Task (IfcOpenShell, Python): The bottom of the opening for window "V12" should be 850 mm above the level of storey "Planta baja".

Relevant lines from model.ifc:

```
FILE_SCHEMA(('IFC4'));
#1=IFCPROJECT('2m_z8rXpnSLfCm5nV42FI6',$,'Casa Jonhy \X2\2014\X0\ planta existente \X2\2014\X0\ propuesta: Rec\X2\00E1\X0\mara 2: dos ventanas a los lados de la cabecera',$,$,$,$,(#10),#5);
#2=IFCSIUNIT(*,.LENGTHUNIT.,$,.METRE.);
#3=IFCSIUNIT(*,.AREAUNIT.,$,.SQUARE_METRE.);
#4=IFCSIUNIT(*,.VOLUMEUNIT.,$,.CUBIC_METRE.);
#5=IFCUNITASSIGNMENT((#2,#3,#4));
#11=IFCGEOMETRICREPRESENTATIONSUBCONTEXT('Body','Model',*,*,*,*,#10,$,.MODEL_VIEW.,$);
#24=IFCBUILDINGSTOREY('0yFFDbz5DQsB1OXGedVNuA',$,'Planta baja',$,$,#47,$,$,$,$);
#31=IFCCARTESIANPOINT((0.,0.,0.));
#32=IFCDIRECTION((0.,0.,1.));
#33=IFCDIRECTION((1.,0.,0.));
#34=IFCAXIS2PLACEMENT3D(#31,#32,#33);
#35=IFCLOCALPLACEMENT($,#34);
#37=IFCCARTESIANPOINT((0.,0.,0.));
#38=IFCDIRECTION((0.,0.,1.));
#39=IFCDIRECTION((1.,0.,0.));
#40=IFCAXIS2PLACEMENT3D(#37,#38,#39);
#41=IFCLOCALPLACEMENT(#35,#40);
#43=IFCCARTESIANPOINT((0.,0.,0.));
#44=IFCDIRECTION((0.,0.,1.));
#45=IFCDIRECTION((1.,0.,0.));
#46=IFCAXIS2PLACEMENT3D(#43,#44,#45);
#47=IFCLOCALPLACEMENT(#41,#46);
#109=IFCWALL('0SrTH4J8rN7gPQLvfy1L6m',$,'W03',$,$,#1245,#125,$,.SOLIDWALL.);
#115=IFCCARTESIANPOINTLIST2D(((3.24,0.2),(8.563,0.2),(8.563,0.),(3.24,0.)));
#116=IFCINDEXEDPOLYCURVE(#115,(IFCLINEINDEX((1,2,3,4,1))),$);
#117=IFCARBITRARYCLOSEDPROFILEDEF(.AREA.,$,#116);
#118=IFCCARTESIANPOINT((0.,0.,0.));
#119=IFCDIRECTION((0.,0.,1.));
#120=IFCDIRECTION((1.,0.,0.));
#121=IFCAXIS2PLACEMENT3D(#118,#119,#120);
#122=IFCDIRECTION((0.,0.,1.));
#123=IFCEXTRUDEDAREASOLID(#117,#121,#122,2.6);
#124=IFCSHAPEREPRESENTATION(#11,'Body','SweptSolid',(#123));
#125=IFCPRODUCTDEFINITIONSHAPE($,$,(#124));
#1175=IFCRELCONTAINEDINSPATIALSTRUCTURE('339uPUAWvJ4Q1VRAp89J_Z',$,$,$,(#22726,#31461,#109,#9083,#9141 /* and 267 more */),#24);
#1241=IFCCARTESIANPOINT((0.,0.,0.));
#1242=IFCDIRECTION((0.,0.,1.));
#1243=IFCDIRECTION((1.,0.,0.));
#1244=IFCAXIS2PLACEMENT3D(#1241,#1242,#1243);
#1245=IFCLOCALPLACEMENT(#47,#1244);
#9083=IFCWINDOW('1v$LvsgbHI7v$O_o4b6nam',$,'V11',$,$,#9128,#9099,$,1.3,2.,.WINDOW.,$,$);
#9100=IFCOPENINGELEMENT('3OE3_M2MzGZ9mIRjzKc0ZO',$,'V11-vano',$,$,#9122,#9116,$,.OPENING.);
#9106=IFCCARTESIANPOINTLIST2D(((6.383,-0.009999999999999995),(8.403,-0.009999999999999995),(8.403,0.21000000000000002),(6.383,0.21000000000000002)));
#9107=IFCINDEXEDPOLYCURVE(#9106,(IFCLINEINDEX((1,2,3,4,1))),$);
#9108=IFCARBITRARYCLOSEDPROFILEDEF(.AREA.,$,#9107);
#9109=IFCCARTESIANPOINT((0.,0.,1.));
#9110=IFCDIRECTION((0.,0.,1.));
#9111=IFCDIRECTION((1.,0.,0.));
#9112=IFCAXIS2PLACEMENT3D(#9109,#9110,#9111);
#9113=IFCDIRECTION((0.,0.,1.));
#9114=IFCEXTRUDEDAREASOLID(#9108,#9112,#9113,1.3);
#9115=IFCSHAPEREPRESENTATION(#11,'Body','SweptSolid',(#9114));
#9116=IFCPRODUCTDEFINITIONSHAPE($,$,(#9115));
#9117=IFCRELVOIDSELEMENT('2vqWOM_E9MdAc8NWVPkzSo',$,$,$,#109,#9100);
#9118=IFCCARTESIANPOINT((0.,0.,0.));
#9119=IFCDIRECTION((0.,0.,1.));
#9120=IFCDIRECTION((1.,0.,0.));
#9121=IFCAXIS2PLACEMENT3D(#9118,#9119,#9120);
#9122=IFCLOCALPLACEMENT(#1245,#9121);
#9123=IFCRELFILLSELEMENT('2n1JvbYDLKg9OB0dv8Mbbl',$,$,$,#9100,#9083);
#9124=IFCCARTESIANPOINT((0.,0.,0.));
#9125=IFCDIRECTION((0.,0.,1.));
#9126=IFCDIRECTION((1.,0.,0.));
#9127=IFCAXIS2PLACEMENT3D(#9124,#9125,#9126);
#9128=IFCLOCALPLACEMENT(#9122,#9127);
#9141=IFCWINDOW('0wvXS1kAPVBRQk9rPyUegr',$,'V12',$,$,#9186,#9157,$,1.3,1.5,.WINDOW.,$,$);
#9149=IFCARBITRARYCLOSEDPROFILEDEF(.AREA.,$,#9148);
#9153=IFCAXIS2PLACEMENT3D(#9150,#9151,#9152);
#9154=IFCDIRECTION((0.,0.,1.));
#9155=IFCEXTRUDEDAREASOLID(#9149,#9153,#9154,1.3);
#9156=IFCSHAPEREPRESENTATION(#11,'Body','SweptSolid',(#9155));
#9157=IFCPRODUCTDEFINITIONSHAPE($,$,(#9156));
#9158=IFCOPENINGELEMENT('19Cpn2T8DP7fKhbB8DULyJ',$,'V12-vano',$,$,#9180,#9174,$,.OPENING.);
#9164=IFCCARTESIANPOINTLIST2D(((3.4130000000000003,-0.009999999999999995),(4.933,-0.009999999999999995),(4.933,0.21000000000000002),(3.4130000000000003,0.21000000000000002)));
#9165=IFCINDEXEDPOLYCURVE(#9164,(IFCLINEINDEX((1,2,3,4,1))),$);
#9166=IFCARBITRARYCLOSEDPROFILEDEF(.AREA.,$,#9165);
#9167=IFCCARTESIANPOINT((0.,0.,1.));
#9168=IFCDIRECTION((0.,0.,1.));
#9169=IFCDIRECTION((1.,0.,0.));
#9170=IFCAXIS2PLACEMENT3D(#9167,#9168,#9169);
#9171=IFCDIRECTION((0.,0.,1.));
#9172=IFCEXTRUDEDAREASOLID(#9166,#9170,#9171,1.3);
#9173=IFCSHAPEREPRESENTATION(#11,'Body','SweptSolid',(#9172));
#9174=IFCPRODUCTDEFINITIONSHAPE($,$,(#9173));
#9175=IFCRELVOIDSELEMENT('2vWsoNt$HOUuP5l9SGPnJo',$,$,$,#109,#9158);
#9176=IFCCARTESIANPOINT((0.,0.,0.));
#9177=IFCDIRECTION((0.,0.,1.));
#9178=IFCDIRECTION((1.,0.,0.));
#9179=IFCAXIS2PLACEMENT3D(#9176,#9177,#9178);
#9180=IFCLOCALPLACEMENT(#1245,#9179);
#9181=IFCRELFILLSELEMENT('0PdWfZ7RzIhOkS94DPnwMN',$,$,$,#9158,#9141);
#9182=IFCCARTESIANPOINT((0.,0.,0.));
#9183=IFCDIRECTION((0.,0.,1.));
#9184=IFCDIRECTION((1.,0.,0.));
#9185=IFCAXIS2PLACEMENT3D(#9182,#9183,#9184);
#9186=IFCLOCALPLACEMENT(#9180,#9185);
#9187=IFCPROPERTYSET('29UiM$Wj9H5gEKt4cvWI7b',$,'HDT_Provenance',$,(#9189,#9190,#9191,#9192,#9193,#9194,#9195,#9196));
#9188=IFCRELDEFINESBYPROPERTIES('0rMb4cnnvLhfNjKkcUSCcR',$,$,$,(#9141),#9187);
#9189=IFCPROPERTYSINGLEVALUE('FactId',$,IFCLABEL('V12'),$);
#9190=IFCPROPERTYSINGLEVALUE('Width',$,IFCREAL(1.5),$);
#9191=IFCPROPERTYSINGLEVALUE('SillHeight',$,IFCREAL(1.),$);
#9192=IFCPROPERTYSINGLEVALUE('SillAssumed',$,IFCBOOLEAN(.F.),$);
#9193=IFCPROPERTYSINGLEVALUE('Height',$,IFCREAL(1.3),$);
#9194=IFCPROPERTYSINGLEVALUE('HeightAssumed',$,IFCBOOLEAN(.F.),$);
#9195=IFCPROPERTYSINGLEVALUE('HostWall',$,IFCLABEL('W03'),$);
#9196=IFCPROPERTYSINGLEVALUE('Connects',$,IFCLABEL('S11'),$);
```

```python
import numpy as np
import ifcopenshell
import ifcopenshell.api.geometry
import ifcopenshell.api.pset
import ifcopenshell.geom
import ifcopenshell.util.element
import ifcopenshell.util.placement
import ifcopenshell.util.shape
import ifcopenshell.util.unit

model = ifcopenshell.open("model.ifc")
unit_scale = ifcopenshell.util.unit.calculate_unit_scale(model)

window = model.by_id(9141)
opening = window.FillsVoids[0].RelatingOpeningElement
storey = ifcopenshell.util.element.get_container(window, ifc_class="IfcBuildingStorey")
level = ifcopenshell.util.placement.get_local_placement(storey.ObjectPlacement)[2, 3]

# The opening's origin need not be at the sill, so measure its lowest point.
shape = ifcopenshell.geom.create_shape(ifcopenshell.geom.settings(), opening)
bottom = ifcopenshell.util.shape.get_shape_bottom_elevation(shape, shape.geometry) / unit_scale
dz = level + 0.85 / unit_scale - bottom

shift = np.array([0.0, 0.0, dz])
# The window is placed relative to its opening, so it follows when the opening moves.
matrix = ifcopenshell.util.placement.get_local_placement(opening.ObjectPlacement)
matrix[:3, 3] += shift
ifcopenshell.api.geometry.edit_object_placement(
    model, product=opening, matrix=matrix, is_si=False, should_transform_children=True
)

# Keep the stored heights in step.
pset = model.by_id(ifcopenshell.util.element.get_pset(window, "HDT_Provenance", should_inherit=False)["id"])
ifcopenshell.api.pset.edit_pset(model, pset=pset, properties={
    "SillHeight": model.create_entity("IfcReal", ifcopenshell.util.element.get_pset(window, "HDT_Provenance", "SillHeight") + dz),
})

print(f"moved by {dz * unit_scale:+.3f} m")

model.write("model_updated.ifc")
```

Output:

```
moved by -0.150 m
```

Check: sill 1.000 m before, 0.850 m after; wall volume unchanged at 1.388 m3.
